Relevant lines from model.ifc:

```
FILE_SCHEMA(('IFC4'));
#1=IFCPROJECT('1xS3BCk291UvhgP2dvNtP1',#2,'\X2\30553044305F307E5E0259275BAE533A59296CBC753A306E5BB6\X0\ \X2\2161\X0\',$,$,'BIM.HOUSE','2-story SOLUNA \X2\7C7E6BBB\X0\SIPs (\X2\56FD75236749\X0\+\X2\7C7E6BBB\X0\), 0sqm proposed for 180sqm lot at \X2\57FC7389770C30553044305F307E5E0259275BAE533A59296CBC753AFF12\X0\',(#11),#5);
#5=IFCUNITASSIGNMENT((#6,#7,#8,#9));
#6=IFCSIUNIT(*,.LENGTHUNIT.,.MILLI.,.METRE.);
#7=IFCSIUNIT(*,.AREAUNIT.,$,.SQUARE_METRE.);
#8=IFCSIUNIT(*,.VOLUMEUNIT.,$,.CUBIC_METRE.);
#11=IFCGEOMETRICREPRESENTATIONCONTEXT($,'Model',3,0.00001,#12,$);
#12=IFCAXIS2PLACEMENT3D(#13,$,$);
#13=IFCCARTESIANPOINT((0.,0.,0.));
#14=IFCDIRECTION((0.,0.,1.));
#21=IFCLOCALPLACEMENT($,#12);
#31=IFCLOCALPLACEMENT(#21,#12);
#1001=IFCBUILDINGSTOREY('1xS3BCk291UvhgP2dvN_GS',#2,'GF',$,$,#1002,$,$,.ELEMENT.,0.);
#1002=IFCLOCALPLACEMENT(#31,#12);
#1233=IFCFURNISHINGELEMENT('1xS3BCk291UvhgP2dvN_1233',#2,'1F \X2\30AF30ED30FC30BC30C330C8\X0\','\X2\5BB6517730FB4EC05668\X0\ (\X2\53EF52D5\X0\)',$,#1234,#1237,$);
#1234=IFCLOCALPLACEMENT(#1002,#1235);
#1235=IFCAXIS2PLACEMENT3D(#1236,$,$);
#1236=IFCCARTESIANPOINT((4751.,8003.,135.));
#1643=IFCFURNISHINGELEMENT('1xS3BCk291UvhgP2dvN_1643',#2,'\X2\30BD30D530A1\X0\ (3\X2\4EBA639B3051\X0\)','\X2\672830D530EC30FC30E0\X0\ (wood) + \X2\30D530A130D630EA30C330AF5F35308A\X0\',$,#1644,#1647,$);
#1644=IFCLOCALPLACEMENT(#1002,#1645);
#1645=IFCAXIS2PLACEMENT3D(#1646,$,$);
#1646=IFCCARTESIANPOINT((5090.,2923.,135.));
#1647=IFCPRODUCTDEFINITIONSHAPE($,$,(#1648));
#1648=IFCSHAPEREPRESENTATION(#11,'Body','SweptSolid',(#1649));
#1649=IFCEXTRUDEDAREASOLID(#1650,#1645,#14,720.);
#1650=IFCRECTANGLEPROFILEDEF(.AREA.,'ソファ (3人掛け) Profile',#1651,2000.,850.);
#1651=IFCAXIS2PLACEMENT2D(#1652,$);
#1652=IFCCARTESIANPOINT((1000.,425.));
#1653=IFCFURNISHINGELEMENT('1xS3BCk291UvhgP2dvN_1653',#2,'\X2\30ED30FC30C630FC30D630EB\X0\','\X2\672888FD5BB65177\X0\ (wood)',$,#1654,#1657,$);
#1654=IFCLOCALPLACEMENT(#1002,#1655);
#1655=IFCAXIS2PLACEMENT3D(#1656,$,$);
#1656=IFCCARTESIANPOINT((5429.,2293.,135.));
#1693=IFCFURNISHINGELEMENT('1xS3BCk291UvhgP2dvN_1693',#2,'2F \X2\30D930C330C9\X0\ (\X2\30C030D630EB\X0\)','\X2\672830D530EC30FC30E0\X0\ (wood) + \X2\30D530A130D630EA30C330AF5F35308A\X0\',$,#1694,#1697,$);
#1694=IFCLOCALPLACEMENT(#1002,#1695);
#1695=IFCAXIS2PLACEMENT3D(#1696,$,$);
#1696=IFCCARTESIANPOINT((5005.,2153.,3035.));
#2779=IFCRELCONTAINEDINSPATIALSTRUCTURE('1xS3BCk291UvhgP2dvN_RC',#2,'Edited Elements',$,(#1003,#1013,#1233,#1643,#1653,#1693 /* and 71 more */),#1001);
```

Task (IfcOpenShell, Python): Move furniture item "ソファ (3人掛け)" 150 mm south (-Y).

```python
import ifcopenshell
import ifcopenshell.api.geometry
import ifcopenshell.util.placement
import ifcopenshell.util.unit

model = ifcopenshell.open("model.ifc")
unit_scale = ifcopenshell.util.unit.calculate_unit_scale(model)

item = model.by_id(1643)
matrix = ifcopenshell.util.placement.get_local_placement(item.ObjectPlacement)
matrix[1, 3] -= 0.15 / unit_scale
ifcopenshell.api.geometry.edit_object_placement(model, product=item, matrix=matrix, is_si=False)

print(ifcopenshell.util.placement.get_local_placement(item.ObjectPlacement).round(3) + 0.0)

model.write("model_rev.ifc")
```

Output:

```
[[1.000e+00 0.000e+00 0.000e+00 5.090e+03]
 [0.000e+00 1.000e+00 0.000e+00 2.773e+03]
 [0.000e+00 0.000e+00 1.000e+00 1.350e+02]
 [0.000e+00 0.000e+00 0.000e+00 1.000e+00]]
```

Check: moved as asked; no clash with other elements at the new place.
